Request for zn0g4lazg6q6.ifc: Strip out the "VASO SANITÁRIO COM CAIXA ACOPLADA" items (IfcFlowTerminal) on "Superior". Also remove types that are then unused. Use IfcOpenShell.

First a look at what the model holds.

```python
import ifcopenshell
import ifcopenshell.util.element

model = ifcopenshell.open("zn0g4lazg6q6.ifc")
print(model.schema)
storey = next(s for s in model.by_type("IfcBuildingStorey") if s.Name == "Superior")
terminals = [e for e in ifcopenshell.util.element.get_decomposition(storey) if e.is_a("IfcFlowTerminal")]
seen = {}
for e in terminals:
    element_type = ifcopenshell.util.element.get_type(e)
    name = element_type.Name if element_type not in (None, e) else None
    seen[name] = seen.get(name, 0) + 1
for name, count in sorted(seen.items(), key=str):
    print(count, "x", name)
```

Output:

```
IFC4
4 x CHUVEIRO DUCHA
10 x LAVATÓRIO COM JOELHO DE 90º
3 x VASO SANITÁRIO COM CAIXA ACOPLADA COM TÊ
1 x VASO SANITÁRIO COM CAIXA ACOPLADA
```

```python
import ifcopenshell
import ifcopenshell.api.root
import ifcopenshell.util.element

model = ifcopenshell.open("zn0g4lazg6q6.ifc")

storey = next(s for s in model.by_type("IfcBuildingStorey") if s.Name == "Superior")
terminals = [e for e in ifcopenshell.util.element.get_decomposition(storey) if e.is_a("IfcFlowTerminal")]
targets = [e for e in terminals if (t := ifcopenshell.util.element.get_type(e)) not in (None, e) and t.Name == "VASO SANITÁRIO COM CAIXA ACOPLADA"]
types = {ifcopenshell.util.element.get_type(e) for e in targets} - {None, *targets}

for e in targets:
    ifcopenshell.api.root.remove_product(model, product=e)
print(len(targets), "removed")

unused = [t for t in types if not ifcopenshell.util.element.get_types(t)]
for t in unused:
    ifcopenshell.api.root.remove_product(model, product=t)
print(len(unused), "unused types removed")

model.write("zn0g4lazg6q6_v2.ifc")
```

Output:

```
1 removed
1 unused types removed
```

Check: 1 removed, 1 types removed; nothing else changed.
